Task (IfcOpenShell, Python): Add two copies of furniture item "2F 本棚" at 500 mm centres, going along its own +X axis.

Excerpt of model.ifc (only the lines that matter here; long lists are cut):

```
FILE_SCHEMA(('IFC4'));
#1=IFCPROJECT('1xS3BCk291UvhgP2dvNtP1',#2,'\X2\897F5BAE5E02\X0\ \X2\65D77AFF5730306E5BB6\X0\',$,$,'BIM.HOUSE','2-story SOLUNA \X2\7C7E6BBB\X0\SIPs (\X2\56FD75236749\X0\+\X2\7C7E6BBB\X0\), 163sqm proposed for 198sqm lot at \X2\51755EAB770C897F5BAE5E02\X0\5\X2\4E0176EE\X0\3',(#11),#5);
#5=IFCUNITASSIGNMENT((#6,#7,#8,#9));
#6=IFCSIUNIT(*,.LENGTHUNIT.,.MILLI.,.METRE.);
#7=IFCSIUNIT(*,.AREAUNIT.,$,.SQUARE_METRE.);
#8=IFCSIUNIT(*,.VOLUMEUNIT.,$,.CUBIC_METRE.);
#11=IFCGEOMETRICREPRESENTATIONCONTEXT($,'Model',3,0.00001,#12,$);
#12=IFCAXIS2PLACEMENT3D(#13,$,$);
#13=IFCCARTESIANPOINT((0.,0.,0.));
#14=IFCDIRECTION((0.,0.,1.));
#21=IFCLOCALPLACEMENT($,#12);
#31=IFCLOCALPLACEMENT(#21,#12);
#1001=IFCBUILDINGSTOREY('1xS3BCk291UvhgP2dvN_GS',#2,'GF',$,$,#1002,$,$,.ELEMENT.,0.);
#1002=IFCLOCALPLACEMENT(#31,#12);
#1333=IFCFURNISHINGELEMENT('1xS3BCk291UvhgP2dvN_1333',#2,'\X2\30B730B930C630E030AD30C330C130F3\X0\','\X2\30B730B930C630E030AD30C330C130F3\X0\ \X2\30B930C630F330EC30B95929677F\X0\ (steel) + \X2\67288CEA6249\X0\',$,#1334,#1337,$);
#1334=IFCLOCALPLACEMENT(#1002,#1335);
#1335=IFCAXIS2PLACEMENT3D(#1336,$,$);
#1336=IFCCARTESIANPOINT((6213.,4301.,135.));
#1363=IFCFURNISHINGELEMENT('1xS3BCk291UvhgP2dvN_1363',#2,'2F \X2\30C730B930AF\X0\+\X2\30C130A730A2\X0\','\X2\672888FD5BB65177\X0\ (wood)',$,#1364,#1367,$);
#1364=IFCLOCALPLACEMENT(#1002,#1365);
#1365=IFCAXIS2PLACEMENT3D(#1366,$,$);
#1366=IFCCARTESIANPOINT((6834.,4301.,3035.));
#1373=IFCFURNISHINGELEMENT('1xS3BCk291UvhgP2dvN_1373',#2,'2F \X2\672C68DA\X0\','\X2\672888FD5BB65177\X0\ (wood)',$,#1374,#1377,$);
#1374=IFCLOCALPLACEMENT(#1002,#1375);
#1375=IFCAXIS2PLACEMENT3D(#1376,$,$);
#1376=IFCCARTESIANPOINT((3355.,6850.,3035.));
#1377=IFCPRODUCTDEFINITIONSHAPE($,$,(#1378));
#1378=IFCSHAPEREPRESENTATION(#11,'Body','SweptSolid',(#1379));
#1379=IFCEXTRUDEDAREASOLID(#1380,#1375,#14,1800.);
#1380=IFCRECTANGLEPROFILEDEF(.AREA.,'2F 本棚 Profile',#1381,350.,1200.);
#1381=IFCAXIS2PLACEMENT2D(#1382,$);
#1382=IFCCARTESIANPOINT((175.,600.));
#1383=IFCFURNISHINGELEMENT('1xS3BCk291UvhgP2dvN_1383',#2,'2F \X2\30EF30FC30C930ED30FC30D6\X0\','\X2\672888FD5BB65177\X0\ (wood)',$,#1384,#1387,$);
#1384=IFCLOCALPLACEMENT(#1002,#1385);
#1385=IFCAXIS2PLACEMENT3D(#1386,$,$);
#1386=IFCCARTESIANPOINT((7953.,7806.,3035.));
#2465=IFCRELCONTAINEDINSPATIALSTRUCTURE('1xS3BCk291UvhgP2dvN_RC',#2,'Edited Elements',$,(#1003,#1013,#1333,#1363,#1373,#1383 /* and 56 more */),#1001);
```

```python
import ifcopenshell
import ifcopenshell.api.geometry
import ifcopenshell.api.root
import ifcopenshell.util.element
import ifcopenshell.util.placement

model = ifcopenshell.open("model.ifc")


def reuse_history(source, copy):
    """copy_class also copies each property set's owner history, people and application; keep the originals."""
    for rel in copy.IsDefinedBy:
        if rel.is_a("IfcRelDefinesByProperties") and (history := rel.RelatingPropertyDefinition.OwnerHistory):
            rel.RelatingPropertyDefinition.OwnerHistory = source.OwnerHistory
            ifcopenshell.util.element.remove_deep2(model, history)


source = model.by_guid("1xS3BCk291UvhgP2dvN_1373")
base = ifcopenshell.util.placement.get_local_placement(source.ObjectPlacement)
step = base[:3, 0] * 500.0

for i in range(1, 3):
    copy = ifcopenshell.api.root.copy_class(model, product=source)
    copy.Representation = ifcopenshell.util.element.copy_deep(
        model, source.Representation, exclude=["IfcGeometricRepresentationContext", "IfcRepresentationMap"]
    )
    reuse_history(source, copy)
    matrix = base.copy()
    matrix[:3, 3] += i * step
    print("added at", matrix[:3, 3].round(3) + 0.0)
    ifcopenshell.api.geometry.edit_object_placement(model, product=copy, matrix=matrix, is_si=False)

model.write("model_rev.ifc")
```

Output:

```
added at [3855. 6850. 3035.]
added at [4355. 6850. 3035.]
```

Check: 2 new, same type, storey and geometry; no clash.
